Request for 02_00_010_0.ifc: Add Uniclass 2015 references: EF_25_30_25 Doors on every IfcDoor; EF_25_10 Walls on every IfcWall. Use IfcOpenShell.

First a look at what the model holds.

```python
import ifcopenshell

model = ifcopenshell.open("02_00_010_0.ifc")
print(model.schema)
print("classifications:", [c.Name for c in model.by_type("IfcClassification")])
for ifc_class in ("IfcDoor", "IfcRoof", "IfcStair", "IfcWall", "IfcWindow"):
    print(ifc_class, len(model.by_type(ifc_class)))
```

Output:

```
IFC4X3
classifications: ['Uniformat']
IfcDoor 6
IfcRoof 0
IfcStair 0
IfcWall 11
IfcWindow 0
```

```python
import ifcopenshell
import ifcopenshell.api.classification

model = ifcopenshell.open("02_00_010_0.ifc")

system = ifcopenshell.api.classification.add_classification(model, classification="Uniclass 2015")

codes = {
    "IfcDoor": ("EF_25_30_25", "Doors"),
    "IfcWall": ("EF_25_10", "Walls"),
}
for ifc_class, (code, name) in codes.items():
    products = model.by_type(ifc_class)
    ifcopenshell.api.classification.add_reference(
        model, products=products, classification=system, identification=code, name=name
    )
    print(code, len(products))

model.write("02_00_010_0_edited.ifc")
```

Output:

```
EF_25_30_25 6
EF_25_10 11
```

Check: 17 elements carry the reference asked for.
